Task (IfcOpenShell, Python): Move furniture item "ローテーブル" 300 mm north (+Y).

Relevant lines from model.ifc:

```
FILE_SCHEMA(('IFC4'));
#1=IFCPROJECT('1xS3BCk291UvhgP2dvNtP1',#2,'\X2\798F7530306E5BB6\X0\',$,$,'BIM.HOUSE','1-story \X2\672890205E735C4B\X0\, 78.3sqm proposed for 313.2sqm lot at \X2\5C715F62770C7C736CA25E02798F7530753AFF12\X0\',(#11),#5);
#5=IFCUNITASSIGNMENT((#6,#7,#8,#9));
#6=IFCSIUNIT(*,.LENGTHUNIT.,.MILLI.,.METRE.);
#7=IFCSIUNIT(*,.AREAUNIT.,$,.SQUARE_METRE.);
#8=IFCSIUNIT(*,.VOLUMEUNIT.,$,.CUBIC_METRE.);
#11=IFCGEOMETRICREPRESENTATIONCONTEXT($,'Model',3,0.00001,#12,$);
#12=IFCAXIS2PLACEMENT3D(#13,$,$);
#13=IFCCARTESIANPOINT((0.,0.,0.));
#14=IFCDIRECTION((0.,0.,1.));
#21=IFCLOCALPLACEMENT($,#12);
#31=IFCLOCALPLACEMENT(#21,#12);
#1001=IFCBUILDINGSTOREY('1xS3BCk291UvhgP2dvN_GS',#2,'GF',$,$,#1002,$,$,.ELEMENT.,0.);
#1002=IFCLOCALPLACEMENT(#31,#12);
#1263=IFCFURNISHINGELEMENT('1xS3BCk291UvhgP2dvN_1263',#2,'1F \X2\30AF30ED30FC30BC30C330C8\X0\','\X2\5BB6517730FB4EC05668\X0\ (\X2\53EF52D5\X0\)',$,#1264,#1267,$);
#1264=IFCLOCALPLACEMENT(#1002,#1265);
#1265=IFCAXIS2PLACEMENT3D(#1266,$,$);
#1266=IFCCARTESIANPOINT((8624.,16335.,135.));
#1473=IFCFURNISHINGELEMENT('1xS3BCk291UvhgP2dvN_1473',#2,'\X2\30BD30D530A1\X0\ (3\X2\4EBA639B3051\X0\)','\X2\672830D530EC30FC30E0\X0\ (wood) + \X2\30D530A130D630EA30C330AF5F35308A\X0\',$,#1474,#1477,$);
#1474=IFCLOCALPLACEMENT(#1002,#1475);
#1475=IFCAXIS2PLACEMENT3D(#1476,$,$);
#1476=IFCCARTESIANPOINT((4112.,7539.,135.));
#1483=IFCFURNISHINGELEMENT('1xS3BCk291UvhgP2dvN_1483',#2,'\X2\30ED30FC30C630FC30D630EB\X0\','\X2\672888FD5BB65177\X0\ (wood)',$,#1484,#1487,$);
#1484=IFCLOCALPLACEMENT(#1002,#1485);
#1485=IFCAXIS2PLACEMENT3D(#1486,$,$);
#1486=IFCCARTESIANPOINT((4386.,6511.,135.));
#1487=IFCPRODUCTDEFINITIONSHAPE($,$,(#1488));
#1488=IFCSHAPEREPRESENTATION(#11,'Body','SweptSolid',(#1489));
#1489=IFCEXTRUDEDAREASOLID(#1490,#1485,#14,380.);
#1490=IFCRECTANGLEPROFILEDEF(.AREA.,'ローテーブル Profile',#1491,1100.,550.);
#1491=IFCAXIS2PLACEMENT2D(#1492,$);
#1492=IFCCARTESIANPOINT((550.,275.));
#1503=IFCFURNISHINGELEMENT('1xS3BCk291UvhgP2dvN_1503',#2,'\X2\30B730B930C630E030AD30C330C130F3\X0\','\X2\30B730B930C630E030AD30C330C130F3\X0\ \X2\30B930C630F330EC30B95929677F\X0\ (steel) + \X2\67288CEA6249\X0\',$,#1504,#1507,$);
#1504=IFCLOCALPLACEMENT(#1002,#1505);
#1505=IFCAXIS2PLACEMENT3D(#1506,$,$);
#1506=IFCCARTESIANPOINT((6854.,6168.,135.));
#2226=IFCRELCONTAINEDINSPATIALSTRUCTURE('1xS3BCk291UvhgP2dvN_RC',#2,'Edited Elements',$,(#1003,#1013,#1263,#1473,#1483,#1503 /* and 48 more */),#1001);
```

```python
import ifcopenshell
import ifcopenshell.api.geometry
import ifcopenshell.util.placement

model = ifcopenshell.open("model.ifc")

item = model.by_guid("1xS3BCk291UvhgP2dvN_1483")
matrix = ifcopenshell.util.placement.get_local_placement(item.ObjectPlacement)
matrix[1, 3] += 300.0
ifcopenshell.api.geometry.edit_object_placement(model, product=item, matrix=matrix, is_si=False)

print(ifcopenshell.util.placement.get_local_placement(item.ObjectPlacement).round(3) + 0.0)

model.write("model_rev.ifc")
```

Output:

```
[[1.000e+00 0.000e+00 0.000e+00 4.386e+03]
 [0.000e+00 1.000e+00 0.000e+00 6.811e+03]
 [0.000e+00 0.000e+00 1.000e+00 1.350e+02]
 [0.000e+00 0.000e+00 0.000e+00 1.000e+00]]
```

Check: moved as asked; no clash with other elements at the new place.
